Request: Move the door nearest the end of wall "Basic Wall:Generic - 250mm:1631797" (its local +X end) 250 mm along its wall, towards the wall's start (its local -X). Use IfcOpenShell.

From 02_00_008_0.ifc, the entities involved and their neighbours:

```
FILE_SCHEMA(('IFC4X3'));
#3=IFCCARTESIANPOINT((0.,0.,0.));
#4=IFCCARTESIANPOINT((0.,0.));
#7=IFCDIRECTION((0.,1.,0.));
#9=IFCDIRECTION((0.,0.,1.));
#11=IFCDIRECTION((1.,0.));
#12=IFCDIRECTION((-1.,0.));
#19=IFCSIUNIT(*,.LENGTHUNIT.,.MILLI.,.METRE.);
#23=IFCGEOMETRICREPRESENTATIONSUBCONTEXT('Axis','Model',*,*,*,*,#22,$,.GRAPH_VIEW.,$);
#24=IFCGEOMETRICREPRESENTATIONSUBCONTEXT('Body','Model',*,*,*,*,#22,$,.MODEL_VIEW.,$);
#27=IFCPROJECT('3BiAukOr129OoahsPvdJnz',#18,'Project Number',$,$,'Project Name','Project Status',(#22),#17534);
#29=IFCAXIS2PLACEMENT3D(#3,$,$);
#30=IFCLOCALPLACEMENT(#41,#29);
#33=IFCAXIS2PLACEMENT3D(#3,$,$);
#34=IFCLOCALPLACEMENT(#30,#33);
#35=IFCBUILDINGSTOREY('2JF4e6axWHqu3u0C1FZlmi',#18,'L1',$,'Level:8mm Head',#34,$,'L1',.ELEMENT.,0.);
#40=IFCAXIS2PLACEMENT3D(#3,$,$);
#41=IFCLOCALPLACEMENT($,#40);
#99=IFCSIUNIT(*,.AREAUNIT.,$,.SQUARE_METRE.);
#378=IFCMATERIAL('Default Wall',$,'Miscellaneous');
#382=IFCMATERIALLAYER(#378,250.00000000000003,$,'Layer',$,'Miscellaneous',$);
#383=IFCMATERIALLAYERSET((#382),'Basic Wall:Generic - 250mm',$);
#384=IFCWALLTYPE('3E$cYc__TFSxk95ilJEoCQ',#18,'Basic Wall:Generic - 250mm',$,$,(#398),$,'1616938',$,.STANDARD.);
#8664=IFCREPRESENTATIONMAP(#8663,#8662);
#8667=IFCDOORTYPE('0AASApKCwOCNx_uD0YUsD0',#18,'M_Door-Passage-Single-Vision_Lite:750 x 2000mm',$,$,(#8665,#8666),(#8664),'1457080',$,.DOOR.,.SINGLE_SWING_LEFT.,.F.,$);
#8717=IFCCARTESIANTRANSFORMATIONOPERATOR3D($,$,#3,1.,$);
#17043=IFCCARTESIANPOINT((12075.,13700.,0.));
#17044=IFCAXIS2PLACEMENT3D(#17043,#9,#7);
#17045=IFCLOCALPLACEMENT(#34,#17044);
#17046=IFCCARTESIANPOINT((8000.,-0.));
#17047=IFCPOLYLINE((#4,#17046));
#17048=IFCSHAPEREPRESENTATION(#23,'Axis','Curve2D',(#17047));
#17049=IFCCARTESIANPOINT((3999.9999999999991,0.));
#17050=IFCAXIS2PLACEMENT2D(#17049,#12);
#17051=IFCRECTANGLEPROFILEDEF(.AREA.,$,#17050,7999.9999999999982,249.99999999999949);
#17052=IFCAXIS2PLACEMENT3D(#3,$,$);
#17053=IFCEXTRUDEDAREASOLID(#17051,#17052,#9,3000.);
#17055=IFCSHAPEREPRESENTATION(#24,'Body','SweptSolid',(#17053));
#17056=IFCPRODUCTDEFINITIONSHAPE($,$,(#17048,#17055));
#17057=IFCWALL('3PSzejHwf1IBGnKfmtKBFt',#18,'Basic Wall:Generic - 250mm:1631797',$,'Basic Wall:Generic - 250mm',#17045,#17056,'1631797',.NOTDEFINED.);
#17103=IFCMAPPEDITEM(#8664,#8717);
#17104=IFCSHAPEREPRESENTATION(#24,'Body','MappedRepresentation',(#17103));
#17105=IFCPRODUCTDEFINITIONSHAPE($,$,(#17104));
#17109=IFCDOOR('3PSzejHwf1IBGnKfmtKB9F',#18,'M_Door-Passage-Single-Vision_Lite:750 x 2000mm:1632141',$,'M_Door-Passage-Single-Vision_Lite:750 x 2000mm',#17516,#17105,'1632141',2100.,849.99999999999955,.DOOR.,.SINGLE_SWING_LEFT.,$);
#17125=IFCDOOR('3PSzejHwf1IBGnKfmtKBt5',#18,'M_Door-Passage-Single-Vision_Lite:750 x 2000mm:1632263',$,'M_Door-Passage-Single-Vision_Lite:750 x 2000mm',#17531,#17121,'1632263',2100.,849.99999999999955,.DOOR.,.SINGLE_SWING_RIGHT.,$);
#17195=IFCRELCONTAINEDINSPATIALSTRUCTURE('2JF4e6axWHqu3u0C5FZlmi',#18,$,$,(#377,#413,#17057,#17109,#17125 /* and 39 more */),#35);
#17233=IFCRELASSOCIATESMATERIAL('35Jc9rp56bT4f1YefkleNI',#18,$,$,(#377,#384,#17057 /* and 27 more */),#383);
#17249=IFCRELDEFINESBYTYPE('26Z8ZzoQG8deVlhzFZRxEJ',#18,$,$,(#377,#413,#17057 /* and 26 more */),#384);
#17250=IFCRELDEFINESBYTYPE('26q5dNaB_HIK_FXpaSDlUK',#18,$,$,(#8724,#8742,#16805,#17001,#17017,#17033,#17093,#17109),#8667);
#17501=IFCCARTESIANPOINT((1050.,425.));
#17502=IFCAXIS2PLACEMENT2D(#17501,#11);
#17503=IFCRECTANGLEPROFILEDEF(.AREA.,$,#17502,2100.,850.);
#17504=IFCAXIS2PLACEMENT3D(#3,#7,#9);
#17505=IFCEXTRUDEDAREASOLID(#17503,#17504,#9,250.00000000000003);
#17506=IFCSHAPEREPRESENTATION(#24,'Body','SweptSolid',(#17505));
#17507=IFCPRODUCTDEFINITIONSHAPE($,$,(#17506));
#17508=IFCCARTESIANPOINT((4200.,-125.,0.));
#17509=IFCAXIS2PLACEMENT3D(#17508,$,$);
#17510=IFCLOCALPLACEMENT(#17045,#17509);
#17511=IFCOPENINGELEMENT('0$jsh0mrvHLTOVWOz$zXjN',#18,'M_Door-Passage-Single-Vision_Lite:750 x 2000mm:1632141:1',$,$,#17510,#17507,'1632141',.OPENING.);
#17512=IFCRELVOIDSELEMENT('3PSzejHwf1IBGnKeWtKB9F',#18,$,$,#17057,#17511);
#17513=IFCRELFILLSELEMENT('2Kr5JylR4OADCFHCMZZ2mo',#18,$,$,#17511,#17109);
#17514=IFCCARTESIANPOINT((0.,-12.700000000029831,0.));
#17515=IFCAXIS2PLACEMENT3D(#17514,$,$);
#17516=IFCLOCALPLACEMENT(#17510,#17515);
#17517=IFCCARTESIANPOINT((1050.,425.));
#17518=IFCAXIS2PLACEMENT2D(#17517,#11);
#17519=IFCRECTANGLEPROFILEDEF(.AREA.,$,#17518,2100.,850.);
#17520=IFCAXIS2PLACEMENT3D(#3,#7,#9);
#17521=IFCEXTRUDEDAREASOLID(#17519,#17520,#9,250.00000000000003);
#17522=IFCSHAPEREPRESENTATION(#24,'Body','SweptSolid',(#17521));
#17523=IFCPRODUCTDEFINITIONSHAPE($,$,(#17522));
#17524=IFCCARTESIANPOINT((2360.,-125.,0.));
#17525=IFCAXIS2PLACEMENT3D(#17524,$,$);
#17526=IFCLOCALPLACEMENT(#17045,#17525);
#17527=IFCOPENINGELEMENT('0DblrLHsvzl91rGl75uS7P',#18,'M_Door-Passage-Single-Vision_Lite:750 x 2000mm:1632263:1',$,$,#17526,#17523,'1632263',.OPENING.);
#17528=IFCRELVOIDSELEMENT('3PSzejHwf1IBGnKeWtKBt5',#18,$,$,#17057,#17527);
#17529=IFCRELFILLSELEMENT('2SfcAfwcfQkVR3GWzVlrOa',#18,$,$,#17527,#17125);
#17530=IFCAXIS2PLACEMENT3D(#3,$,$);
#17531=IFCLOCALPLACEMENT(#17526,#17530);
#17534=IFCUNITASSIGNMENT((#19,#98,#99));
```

```python
import ifcopenshell
import ifcopenshell.api.geometry
import ifcopenshell.util.placement
import ifcopenshell.util.unit

model = ifcopenshell.open("02_00_008_0.ifc")
unit_scale = ifcopenshell.util.unit.calculate_unit_scale(model)

door = model.by_id(17109)
opening = door.FillsVoids[0].RelatingOpeningElement
wall = opening.VoidsElements[0].RelatingBuildingElement

wall_matrix = ifcopenshell.util.placement.get_local_placement(wall.ObjectPlacement)
shift = wall_matrix[:3, 0] * -0.25 / unit_scale
before = ifcopenshell.util.placement.get_local_placement(door.ObjectPlacement)[:3, 3].copy()

# The door is placed relative to its opening, so it follows when the opening moves.
matrix = ifcopenshell.util.placement.get_local_placement(opening.ObjectPlacement)
matrix[:3, 3] += shift
ifcopenshell.api.geometry.edit_object_placement(
    model, product=opening, matrix=matrix, is_si=False, should_transform_children=True
)

after = ifcopenshell.util.placement.get_local_placement(door.ObjectPlacement)[:3, 3]
print("door moved by", (after - before).round(3) + 0.0)

model.write("02_00_008_0_updated.ifc")
```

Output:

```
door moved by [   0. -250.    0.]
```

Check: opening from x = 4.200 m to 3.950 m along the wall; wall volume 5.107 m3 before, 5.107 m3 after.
